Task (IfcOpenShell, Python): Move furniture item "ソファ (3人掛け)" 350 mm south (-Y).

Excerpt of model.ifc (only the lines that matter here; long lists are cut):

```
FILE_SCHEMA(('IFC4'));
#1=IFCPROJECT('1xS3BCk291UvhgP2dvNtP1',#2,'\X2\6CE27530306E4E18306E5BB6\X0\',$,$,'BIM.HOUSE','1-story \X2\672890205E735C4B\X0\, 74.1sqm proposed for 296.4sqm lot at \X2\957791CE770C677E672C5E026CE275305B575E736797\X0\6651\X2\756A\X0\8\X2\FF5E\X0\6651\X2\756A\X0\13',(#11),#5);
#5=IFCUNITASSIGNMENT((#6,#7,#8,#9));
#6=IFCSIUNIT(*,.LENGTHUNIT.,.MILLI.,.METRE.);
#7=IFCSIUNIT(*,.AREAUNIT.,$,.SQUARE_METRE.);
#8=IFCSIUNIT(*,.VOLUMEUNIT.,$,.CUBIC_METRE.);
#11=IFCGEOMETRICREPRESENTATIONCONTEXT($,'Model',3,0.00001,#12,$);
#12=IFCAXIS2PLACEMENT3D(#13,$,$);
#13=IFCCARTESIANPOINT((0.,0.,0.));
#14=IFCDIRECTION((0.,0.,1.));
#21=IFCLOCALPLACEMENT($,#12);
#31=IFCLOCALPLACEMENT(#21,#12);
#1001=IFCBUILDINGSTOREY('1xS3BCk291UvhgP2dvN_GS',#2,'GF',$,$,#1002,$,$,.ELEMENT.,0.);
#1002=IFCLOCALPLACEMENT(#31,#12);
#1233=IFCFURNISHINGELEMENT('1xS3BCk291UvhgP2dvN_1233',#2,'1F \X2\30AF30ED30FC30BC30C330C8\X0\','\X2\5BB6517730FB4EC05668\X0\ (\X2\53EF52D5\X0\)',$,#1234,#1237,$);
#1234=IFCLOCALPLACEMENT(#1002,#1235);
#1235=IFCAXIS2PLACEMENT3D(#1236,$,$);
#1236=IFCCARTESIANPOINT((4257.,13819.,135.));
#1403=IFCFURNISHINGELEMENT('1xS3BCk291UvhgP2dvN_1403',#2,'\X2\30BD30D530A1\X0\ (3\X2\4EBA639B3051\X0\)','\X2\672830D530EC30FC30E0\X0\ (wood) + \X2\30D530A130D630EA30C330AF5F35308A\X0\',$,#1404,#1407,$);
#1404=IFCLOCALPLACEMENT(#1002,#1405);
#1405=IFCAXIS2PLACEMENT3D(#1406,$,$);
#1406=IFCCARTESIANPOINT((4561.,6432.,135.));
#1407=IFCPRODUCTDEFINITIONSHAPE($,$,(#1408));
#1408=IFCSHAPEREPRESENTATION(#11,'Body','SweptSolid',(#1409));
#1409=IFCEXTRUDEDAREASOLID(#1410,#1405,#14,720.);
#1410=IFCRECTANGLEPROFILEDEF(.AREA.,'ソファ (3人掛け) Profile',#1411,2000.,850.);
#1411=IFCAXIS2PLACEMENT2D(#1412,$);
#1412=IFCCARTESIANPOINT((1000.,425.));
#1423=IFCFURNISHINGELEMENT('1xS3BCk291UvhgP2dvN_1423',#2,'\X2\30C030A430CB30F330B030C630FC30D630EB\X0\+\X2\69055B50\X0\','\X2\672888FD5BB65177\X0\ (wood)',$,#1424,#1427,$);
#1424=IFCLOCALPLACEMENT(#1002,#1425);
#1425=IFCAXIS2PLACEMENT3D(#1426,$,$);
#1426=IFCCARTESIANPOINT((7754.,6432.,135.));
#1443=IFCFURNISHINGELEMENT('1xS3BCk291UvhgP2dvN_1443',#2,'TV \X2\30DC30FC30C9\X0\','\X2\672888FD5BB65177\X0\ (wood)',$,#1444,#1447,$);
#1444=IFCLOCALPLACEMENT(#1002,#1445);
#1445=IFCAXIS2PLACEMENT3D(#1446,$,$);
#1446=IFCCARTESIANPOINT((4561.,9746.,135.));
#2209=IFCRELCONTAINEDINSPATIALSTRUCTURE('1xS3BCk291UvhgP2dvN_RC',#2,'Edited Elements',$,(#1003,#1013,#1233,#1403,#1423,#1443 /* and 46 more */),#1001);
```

```python
import ifcopenshell
import ifcopenshell.api.geometry
import ifcopenshell.util.placement

model = ifcopenshell.open("model.ifc")

item = model.by_guid("1xS3BCk291UvhgP2dvN_1403")
matrix = ifcopenshell.util.placement.get_local_placement(item.ObjectPlacement)
matrix[1, 3] -= 350.0
ifcopenshell.api.geometry.edit_object_placement(model, product=item, matrix=matrix, is_si=False)

print(ifcopenshell.util.placement.get_local_placement(item.ObjectPlacement).round(3) + 0.0)

model.write("model_edited.ifc")
```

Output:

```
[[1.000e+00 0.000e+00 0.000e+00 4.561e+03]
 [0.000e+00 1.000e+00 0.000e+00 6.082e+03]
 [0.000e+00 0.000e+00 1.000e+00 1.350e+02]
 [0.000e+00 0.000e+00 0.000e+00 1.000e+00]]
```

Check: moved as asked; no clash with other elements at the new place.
